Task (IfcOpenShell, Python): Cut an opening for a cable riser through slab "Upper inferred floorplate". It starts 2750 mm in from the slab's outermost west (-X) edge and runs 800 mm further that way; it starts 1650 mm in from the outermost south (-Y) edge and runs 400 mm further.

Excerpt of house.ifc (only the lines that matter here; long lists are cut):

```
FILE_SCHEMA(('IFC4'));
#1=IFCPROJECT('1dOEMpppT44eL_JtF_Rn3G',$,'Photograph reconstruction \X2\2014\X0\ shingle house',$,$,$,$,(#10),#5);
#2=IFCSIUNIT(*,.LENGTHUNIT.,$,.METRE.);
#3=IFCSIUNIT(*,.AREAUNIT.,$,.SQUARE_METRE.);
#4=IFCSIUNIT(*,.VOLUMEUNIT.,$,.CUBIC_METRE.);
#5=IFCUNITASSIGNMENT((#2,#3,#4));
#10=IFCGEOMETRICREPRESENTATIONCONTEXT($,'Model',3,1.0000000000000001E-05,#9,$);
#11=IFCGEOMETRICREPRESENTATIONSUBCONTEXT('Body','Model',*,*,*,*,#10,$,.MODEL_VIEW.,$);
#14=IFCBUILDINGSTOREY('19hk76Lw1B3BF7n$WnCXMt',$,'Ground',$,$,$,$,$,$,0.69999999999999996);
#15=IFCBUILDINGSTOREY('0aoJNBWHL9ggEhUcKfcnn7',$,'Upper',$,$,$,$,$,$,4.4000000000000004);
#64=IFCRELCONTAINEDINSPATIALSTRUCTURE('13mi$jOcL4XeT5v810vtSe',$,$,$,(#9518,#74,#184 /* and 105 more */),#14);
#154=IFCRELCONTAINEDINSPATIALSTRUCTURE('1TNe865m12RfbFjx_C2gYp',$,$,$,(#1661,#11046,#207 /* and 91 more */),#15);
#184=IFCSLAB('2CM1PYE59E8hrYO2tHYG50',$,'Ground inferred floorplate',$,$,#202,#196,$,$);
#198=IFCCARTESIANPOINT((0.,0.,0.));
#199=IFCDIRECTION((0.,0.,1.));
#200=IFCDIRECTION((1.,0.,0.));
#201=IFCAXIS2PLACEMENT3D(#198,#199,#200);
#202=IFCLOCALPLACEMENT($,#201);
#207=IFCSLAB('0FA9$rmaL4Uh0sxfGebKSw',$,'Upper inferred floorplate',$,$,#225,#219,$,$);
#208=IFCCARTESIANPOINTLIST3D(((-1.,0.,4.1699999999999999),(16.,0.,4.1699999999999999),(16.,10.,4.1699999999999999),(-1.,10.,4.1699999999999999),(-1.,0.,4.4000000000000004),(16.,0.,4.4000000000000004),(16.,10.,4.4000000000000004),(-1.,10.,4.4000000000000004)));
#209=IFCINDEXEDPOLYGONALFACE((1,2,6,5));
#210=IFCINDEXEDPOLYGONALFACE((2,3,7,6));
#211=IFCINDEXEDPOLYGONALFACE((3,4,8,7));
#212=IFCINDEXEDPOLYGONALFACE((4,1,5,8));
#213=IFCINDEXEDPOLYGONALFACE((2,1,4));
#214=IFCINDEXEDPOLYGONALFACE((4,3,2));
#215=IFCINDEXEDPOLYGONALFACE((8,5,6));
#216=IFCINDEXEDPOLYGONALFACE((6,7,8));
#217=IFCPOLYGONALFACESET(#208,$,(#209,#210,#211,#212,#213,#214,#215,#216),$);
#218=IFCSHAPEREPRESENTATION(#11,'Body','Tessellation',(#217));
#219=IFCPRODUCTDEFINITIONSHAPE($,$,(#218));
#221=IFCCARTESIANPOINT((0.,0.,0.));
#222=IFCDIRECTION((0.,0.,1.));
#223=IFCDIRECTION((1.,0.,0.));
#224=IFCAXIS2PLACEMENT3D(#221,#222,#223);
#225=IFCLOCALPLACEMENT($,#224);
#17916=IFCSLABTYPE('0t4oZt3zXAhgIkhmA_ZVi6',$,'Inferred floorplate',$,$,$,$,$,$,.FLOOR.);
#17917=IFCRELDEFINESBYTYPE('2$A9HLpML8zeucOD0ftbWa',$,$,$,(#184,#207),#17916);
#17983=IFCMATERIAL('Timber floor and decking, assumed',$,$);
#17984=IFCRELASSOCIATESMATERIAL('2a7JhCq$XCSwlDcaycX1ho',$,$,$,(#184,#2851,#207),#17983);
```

```python
import numpy as np
import ifcopenshell
import ifcopenshell.api.feature
import ifcopenshell.api.geometry
import ifcopenshell.api.root
import ifcopenshell.geom
import ifcopenshell.util.placement
import ifcopenshell.util.representation
import ifcopenshell.util.shape
import ifcopenshell.util.unit

model = ifcopenshell.open("house.ifc")
unit_scale = ifcopenshell.util.unit.calculate_unit_scale(model)
settings = ifcopenshell.geom.settings()


def volume(element):
    """Net volume in cubic metres, openings subtracted."""
    shape = ifcopenshell.geom.create_shape(settings, element)
    return ifcopenshell.util.shape.get_volume(shape.geometry)


slab = model.by_guid("0FA9$rmaL4Uh0sxfGebKSw")
before = volume(slab)

# Extent in the slab's own axes, in metres. The edges named are its -X and -Y sides.
slab_shape = ifcopenshell.geom.create_shape(settings, slab)
vertices = ifcopenshell.util.shape.get_vertices(slab_shape.geometry)
x_min, y_min, bottom = vertices.min(axis=0)
top = vertices[:, 2].max()

opening = ifcopenshell.api.root.create_entity(model, ifc_class="IfcOpeningElement", name="Cable riser opening", predefined_type="OPENING")
context = ifcopenshell.util.representation.get_context(model, "Model", "Body", "MODEL_VIEW")
width, depth = 0.8, 0.4
outline = [(0.0, 0.0), (width, 0.0), (width, depth), (0.0, depth), (0.0, 0.0)]
# Overshoot both faces by 50 mm so the cut is clean.
shape = ifcopenshell.api.geometry.add_slab_representation(
    model, context=context, depth=top - bottom + 0.1, polyline=outline
)
ifcopenshell.api.geometry.assign_representation(model, product=opening, representation=shape)

matrix = ifcopenshell.util.placement.get_local_placement(slab.ObjectPlacement)
matrix[:, 3] = matrix @ np.append(np.array([x_min + 2.75, y_min + 1.65, bottom - 0.05]) / unit_scale, 1.0)
ifcopenshell.api.geometry.edit_object_placement(model, product=opening, matrix=matrix, is_si=False)
ifcopenshell.api.feature.add_feature(model, feature=opening, element=slab)

after = volume(slab)

print(f"slab volume {before:.3f} -> {after:.3f} m3")

model.write("house-out.ifc")
```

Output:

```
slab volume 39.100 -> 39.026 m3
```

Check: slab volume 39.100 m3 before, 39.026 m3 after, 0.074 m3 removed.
